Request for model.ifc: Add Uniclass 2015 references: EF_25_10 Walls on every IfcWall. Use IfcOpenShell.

First a look at what the model holds.

```python
import ifcopenshell

model = ifcopenshell.open("model.ifc")
print(model.schema)
print("classifications:", [c.Name for c in model.by_type("IfcClassification")])
for ifc_class in ("IfcDoor", "IfcRoof", "IfcStair", "IfcWall", "IfcWindow"):
    print(ifc_class, len(model.by_type(ifc_class)))
```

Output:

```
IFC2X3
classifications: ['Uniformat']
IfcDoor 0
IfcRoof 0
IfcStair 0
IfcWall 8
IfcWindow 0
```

```python
import ifcopenshell
import ifcopenshell.api.classification

model = ifcopenshell.open("model.ifc")

# IFC2X3 requires Source and Edition and has no link from the project to the system.
system = model.create_entity("IfcClassification", Source="NBS", Edition="2015", Name="Uniclass 2015")

codes = {
    "IfcWall": ("EF_25_10", "Walls"),
}
for ifc_class, (code, name) in codes.items():
    products = model.by_type(ifc_class)
    ifcopenshell.api.classification.add_reference(
        model, products=products, classification=system, identification=code, name=name
    )
    print(code, len(products))

model.write("model_rev.ifc")
```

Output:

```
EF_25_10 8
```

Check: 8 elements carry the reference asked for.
